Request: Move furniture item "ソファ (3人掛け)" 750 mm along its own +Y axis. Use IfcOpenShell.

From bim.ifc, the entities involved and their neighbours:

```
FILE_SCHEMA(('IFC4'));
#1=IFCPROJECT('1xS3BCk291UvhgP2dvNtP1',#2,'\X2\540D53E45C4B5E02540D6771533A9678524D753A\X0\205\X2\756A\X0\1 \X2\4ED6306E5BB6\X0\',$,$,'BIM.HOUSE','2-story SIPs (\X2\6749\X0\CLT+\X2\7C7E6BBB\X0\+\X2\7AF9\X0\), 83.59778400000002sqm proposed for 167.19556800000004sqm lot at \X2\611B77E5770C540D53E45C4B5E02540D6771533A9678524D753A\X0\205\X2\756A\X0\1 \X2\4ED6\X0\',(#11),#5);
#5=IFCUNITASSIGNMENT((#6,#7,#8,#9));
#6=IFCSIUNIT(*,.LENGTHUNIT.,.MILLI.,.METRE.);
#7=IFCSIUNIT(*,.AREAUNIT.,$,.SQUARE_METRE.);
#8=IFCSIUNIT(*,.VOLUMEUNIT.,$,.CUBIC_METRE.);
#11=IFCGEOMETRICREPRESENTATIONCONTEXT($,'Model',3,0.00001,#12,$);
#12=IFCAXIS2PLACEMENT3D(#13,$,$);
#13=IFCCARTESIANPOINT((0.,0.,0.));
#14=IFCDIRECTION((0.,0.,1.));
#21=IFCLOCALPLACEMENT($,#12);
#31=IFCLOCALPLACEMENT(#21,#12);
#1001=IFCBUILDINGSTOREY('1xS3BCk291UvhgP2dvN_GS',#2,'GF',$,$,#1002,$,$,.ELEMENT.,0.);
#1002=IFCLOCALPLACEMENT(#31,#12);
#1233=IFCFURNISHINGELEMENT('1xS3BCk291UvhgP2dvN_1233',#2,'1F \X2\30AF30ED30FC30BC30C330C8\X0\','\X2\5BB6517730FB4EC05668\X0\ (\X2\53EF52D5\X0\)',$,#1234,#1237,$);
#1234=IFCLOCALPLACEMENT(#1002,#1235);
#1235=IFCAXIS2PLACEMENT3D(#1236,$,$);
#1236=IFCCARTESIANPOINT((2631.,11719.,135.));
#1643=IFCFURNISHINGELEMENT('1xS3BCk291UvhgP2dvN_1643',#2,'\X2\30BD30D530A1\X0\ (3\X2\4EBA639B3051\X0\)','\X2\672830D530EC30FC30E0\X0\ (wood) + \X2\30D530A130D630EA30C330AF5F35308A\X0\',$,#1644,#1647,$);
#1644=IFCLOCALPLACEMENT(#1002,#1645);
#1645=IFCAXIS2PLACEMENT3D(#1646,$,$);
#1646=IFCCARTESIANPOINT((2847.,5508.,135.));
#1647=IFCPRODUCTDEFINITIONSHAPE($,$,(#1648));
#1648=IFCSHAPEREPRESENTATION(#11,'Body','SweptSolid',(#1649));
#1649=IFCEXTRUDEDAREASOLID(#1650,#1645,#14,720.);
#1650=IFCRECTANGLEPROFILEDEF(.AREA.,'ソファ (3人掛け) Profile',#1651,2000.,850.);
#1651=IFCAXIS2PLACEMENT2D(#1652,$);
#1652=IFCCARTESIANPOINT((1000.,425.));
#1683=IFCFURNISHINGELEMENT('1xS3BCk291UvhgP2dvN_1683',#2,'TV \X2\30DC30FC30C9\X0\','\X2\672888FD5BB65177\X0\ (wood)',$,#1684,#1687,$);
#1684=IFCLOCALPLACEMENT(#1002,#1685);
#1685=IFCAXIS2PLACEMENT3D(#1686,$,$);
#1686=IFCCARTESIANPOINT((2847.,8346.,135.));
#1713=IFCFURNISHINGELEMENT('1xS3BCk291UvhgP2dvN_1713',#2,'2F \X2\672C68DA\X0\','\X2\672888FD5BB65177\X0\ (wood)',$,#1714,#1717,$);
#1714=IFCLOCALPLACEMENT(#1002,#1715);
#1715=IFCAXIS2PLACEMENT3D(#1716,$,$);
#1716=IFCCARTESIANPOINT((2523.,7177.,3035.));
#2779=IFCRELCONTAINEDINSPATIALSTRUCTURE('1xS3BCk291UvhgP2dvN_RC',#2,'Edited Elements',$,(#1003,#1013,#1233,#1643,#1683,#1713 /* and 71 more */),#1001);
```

```python
import ifcopenshell
import ifcopenshell.api.geometry
import ifcopenshell.util.placement
import ifcopenshell.util.unit

model = ifcopenshell.open("bim.ifc")
unit_scale = ifcopenshell.util.unit.calculate_unit_scale(model)

item = model.by_guid("1xS3BCk291UvhgP2dvN_1643")
matrix = ifcopenshell.util.placement.get_local_placement(item.ObjectPlacement)
matrix[:3, 3] += matrix[:3, 1] * 0.75 / unit_scale
ifcopenshell.api.geometry.edit_object_placement(model, product=item, matrix=matrix, is_si=False)

print(ifcopenshell.util.placement.get_local_placement(item.ObjectPlacement).round(3) + 0.0)

model.write("bim_rev.ifc")
```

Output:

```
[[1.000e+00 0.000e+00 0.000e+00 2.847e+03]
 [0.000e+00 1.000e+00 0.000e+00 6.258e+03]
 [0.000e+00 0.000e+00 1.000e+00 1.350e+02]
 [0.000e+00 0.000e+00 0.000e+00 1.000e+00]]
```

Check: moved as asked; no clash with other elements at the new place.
